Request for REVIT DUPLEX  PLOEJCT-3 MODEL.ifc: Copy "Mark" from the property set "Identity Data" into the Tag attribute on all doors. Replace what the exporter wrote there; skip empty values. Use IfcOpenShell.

First a look at what the model holds.

```python
import ifcopenshell
import ifcopenshell.util.element

model = ifcopenshell.open("REVIT DUPLEX  PLOEJCT-3 MODEL.ifc")
print(model.schema)
doors = model.by_type("IfcDoor")
print(len(doors), "doors")
for e in doors[:8]:
    source = ifcopenshell.util.element.get_pset(e, "Identity Data", "Mark")
    target = e.Tag
    print(e.id(), repr(source), repr(target), sep=" | ")
```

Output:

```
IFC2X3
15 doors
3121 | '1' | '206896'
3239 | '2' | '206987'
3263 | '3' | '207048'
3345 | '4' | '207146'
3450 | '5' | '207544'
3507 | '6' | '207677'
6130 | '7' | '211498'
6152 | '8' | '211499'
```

```python
import ifcopenshell
import ifcopenshell.util.element

model = ifcopenshell.open("REVIT DUPLEX  PLOEJCT-3 MODEL.ifc")

count = 0
for e in model.by_type("IfcDoor"):
    value = ifcopenshell.util.element.get_pset(e, "Identity Data", "Mark")
    current = e.Tag
    if not value or not value.strip() or current == value:
        continue
    e.Tag = value
    count += 1

print(count, "doors updated")

model.write("REVIT DUPLEX  PLOEJCT-3 MODEL-out.ifc")
```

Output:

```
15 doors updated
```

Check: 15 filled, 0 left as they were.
